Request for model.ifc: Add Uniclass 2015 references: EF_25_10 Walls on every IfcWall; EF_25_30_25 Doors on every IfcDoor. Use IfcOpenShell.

First a look at what the model holds.

```python
import ifcopenshell

model = ifcopenshell.open("model.ifc")
print(model.schema)
print("classifications:", [c.Name for c in model.by_type("IfcClassification")])
for ifc_class in ("IfcDoor", "IfcRoof", "IfcStair", "IfcWall", "IfcWindow"):
    print(ifc_class, len(model.by_type(ifc_class)))
```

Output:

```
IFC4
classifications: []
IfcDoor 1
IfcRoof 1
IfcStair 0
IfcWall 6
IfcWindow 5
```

```python
import ifcopenshell
import ifcopenshell.api.classification

model = ifcopenshell.open("model.ifc")

system = ifcopenshell.api.classification.add_classification(model, classification="Uniclass 2015")

codes = {
    "IfcWall": ("EF_25_10", "Walls"),
    "IfcDoor": ("EF_25_30_25", "Doors"),
}
for ifc_class, (code, name) in codes.items():
    products = model.by_type(ifc_class)
    ifcopenshell.api.classification.add_reference(
        model, products=products, classification=system, identification=code, name=name
    )
    print(code, len(products))

model.write("model-out.ifc")
```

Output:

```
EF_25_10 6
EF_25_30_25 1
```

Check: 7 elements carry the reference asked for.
